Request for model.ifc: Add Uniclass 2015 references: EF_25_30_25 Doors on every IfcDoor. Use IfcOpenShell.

First a look at what the model holds.

```python
import ifcopenshell

model = ifcopenshell.open("model.ifc")
print(model.schema)
print("classifications:", [c.Name for c in model.by_type("IfcClassification")])
for ifc_class in ("IfcDoor", "IfcRoof", "IfcStair", "IfcWall", "IfcWindow"):
    print(ifc_class, len(model.by_type(ifc_class)))
```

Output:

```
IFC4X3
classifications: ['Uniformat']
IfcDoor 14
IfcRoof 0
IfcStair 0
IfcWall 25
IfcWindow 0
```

```python
import ifcopenshell
import ifcopenshell.api.classification

model = ifcopenshell.open("model.ifc")

system = ifcopenshell.api.classification.add_classification(model, classification="Uniclass 2015")

codes = {
    "IfcDoor": ("EF_25_30_25", "Doors"),
}
for ifc_class, (code, name) in codes.items():
    products = model.by_type(ifc_class)
    ifcopenshell.api.classification.add_reference(
        model, products=products, classification=system, identification=code, name=name
    )
    print(code, len(products))

model.write("model-out.ifc")
```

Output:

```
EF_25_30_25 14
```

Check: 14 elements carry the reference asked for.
